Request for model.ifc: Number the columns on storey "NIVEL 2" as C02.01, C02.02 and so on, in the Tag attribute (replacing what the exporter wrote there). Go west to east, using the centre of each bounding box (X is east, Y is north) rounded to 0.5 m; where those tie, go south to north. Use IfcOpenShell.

First a look at what the model holds.

```python
import ifcopenshell
import ifcopenshell.util.element
import ifcopenshell.util.placement

model = ifcopenshell.open("model.ifc")
print(model.schema)
storey = next(s for s in model.by_type("IfcBuildingStorey") if s.Name == "NIVEL 2")
columns = [e for e in ifcopenshell.util.element.get_decomposition(storey) if e.is_a("IfcColumn")]
for e in sorted(columns, key=lambda e: e.id()):
    origin = ifcopenshell.util.placement.get_local_placement(e.ObjectPlacement)[:3, 3]
    print(e.id(), e.Tag, e.Name, origin.round(2) + 0.0, sep=" | ")
```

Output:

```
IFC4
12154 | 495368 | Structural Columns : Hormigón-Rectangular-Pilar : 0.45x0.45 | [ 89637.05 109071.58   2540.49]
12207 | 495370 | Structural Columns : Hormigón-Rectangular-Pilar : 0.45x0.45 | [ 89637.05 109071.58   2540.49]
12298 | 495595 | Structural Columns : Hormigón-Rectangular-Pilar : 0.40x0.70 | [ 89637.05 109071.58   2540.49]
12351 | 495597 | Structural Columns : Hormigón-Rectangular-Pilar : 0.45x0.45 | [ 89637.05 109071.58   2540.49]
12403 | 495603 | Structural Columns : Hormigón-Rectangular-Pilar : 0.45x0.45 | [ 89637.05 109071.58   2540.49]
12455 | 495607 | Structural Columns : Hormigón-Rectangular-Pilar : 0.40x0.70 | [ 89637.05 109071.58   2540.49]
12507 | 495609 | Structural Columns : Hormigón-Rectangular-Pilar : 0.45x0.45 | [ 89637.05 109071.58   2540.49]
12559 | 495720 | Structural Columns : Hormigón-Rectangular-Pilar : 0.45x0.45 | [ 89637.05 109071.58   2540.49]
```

```python
import ifcopenshell
import ifcopenshell.geom
import ifcopenshell.util.element
import ifcopenshell.util.shape

model = ifcopenshell.open("model.ifc")
settings = ifcopenshell.geom.settings()
settings.set("use-world-coords", True)


def centre(element):
    shape = ifcopenshell.geom.create_shape(settings, element)
    return ifcopenshell.util.shape.get_bbox_centroid(shape.geometry)


storey = next(s for s in model.by_type("IfcBuildingStorey") if s.Name == "NIVEL 2")
columns = [e for e in ifcopenshell.util.element.get_decomposition(storey) if e.is_a("IfcColumn")]

# Insertion points can sit at a corner or the storey origin, so sort by the geometry (in metres).
centres = {e: centre(e) for e in columns}
columns.sort(key=lambda e: (round(centres[e][0] / 0.5), centres[e][1]))

for i, e in enumerate(columns, start=1):
    number = f"C02.{i:02d}"
    e.Tag = number
    print(e.id(), number)

model.write("model_rev.ifc")
```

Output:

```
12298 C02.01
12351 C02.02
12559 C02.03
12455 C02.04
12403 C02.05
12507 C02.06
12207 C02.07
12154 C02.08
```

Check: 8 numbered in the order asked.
